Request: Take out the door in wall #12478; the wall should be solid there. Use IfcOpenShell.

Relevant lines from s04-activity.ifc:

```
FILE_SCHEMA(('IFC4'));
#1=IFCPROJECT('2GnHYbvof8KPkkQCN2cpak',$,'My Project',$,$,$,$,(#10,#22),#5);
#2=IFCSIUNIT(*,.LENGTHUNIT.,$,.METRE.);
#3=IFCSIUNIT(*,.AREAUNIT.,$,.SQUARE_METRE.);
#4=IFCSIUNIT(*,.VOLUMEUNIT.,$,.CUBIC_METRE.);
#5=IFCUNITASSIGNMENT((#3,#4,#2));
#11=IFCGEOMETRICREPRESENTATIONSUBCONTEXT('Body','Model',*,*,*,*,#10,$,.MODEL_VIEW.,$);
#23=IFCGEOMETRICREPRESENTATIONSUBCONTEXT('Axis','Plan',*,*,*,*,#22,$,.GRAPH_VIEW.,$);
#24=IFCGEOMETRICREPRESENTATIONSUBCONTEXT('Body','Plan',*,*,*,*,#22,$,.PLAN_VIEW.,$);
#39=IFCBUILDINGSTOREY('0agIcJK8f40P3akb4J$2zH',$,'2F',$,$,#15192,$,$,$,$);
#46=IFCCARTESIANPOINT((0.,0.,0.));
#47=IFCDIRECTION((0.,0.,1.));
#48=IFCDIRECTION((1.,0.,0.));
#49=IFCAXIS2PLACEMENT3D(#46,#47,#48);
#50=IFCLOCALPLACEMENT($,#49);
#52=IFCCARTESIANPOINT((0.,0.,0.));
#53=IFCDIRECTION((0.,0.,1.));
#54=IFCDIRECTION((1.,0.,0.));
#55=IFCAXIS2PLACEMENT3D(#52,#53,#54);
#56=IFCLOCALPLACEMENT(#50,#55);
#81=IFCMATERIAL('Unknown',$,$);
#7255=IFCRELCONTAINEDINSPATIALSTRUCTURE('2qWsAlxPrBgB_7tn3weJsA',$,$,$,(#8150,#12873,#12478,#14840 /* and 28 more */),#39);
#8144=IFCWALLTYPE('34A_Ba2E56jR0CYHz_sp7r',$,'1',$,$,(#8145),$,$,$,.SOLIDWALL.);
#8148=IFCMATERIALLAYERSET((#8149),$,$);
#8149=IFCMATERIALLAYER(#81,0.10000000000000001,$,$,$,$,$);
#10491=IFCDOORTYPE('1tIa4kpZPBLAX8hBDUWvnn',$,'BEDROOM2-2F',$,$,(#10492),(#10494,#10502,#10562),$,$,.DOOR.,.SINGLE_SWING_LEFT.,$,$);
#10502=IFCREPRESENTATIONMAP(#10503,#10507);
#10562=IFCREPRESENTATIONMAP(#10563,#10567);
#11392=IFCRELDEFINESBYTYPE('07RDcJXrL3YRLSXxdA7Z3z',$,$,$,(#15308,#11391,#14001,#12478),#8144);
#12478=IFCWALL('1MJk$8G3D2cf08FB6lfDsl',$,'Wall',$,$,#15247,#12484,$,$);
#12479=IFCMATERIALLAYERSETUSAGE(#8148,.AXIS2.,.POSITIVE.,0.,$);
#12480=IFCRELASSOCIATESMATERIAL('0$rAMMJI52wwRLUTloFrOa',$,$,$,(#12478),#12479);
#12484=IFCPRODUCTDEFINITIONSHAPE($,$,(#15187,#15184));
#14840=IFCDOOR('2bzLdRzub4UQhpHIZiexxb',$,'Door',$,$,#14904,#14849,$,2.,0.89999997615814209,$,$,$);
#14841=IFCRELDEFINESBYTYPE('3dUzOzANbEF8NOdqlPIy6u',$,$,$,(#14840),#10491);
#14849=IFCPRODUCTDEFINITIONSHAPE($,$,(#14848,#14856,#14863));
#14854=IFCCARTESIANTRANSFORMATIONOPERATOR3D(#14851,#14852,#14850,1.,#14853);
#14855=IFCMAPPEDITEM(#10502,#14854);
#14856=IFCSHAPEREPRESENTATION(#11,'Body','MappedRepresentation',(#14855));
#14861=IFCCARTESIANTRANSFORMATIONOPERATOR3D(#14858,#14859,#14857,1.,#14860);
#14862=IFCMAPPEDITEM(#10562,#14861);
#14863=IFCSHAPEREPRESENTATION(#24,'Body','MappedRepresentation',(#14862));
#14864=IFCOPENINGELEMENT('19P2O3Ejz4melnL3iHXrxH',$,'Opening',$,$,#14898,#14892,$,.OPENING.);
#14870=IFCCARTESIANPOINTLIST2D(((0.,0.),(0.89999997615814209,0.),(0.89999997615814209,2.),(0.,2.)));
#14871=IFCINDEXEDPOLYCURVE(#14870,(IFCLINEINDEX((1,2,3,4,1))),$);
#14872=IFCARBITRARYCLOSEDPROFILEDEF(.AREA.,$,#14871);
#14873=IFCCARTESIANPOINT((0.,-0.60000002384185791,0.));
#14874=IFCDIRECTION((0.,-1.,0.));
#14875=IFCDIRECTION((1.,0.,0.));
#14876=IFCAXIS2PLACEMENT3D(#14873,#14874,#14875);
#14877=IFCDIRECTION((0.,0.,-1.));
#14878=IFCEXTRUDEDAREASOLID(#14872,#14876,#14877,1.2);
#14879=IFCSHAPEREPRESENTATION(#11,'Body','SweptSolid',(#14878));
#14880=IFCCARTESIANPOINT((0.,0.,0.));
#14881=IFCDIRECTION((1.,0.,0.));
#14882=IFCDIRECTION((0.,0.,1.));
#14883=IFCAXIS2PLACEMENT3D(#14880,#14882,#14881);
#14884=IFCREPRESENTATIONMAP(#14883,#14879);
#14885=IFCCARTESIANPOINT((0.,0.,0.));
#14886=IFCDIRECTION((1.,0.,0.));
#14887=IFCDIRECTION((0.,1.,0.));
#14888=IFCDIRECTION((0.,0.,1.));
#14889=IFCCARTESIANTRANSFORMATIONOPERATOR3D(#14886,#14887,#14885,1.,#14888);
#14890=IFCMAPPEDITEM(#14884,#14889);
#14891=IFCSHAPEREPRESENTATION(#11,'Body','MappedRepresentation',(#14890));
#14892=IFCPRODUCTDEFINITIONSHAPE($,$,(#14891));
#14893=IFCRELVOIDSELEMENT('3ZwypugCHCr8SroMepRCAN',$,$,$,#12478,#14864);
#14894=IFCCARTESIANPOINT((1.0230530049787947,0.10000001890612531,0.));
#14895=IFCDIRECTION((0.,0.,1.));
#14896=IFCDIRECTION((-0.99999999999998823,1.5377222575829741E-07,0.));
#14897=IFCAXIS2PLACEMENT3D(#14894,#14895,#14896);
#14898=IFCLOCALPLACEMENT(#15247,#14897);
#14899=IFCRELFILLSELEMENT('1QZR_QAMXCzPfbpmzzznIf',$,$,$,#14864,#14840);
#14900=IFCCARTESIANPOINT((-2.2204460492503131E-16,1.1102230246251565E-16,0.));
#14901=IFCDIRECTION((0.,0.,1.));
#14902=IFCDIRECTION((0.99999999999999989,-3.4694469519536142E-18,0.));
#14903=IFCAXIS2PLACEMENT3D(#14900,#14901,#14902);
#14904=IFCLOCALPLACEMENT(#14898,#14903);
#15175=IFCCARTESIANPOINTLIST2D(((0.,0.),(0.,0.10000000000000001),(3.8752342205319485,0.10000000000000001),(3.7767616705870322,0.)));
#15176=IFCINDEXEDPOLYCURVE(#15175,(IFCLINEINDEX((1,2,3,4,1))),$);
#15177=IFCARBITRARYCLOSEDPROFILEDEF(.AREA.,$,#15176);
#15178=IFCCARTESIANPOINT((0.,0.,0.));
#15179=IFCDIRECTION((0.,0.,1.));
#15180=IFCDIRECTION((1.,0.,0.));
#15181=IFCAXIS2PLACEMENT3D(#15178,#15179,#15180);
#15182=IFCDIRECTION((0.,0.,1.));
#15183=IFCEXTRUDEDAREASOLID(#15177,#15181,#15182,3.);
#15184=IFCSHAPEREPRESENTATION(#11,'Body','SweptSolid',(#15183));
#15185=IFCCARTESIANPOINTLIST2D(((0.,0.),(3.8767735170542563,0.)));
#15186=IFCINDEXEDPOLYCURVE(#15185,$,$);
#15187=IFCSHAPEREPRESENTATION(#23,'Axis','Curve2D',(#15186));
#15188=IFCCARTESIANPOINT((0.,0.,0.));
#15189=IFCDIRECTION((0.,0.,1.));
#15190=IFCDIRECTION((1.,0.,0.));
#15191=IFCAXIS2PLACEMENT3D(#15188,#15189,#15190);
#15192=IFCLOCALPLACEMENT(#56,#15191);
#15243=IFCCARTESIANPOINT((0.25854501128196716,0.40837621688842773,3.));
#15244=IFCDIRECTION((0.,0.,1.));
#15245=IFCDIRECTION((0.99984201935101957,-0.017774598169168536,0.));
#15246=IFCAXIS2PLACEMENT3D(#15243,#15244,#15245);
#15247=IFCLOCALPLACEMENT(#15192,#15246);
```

```python
import ifcopenshell
import ifcopenshell.api.feature
import ifcopenshell.api.root
import ifcopenshell.geom
import ifcopenshell.util.shape

model = ifcopenshell.open("s04-activity.ifc")
settings = ifcopenshell.geom.settings()


def volume(element):
    """Net volume in cubic metres, openings subtracted."""
    shape = ifcopenshell.geom.create_shape(settings, element)
    return ifcopenshell.util.shape.get_volume(shape.geometry)


door = model.by_guid("2bzLdRzub4UQhpHIZiexxb")
opening = door.FillsVoids[0].RelatingOpeningElement
wall = opening.VoidsElements[0].RelatingBuildingElement
before = volume(wall)

ifcopenshell.api.root.remove_product(model, product=door)
ifcopenshell.api.feature.remove_feature(model, feature=opening)

after = volume(wall)

print(f"wall volume {before:.3f} -> {after:.3f} m3")

model.write("s04-activity_edited.ifc")
```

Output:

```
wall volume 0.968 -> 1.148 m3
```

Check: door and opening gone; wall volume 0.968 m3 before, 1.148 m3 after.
